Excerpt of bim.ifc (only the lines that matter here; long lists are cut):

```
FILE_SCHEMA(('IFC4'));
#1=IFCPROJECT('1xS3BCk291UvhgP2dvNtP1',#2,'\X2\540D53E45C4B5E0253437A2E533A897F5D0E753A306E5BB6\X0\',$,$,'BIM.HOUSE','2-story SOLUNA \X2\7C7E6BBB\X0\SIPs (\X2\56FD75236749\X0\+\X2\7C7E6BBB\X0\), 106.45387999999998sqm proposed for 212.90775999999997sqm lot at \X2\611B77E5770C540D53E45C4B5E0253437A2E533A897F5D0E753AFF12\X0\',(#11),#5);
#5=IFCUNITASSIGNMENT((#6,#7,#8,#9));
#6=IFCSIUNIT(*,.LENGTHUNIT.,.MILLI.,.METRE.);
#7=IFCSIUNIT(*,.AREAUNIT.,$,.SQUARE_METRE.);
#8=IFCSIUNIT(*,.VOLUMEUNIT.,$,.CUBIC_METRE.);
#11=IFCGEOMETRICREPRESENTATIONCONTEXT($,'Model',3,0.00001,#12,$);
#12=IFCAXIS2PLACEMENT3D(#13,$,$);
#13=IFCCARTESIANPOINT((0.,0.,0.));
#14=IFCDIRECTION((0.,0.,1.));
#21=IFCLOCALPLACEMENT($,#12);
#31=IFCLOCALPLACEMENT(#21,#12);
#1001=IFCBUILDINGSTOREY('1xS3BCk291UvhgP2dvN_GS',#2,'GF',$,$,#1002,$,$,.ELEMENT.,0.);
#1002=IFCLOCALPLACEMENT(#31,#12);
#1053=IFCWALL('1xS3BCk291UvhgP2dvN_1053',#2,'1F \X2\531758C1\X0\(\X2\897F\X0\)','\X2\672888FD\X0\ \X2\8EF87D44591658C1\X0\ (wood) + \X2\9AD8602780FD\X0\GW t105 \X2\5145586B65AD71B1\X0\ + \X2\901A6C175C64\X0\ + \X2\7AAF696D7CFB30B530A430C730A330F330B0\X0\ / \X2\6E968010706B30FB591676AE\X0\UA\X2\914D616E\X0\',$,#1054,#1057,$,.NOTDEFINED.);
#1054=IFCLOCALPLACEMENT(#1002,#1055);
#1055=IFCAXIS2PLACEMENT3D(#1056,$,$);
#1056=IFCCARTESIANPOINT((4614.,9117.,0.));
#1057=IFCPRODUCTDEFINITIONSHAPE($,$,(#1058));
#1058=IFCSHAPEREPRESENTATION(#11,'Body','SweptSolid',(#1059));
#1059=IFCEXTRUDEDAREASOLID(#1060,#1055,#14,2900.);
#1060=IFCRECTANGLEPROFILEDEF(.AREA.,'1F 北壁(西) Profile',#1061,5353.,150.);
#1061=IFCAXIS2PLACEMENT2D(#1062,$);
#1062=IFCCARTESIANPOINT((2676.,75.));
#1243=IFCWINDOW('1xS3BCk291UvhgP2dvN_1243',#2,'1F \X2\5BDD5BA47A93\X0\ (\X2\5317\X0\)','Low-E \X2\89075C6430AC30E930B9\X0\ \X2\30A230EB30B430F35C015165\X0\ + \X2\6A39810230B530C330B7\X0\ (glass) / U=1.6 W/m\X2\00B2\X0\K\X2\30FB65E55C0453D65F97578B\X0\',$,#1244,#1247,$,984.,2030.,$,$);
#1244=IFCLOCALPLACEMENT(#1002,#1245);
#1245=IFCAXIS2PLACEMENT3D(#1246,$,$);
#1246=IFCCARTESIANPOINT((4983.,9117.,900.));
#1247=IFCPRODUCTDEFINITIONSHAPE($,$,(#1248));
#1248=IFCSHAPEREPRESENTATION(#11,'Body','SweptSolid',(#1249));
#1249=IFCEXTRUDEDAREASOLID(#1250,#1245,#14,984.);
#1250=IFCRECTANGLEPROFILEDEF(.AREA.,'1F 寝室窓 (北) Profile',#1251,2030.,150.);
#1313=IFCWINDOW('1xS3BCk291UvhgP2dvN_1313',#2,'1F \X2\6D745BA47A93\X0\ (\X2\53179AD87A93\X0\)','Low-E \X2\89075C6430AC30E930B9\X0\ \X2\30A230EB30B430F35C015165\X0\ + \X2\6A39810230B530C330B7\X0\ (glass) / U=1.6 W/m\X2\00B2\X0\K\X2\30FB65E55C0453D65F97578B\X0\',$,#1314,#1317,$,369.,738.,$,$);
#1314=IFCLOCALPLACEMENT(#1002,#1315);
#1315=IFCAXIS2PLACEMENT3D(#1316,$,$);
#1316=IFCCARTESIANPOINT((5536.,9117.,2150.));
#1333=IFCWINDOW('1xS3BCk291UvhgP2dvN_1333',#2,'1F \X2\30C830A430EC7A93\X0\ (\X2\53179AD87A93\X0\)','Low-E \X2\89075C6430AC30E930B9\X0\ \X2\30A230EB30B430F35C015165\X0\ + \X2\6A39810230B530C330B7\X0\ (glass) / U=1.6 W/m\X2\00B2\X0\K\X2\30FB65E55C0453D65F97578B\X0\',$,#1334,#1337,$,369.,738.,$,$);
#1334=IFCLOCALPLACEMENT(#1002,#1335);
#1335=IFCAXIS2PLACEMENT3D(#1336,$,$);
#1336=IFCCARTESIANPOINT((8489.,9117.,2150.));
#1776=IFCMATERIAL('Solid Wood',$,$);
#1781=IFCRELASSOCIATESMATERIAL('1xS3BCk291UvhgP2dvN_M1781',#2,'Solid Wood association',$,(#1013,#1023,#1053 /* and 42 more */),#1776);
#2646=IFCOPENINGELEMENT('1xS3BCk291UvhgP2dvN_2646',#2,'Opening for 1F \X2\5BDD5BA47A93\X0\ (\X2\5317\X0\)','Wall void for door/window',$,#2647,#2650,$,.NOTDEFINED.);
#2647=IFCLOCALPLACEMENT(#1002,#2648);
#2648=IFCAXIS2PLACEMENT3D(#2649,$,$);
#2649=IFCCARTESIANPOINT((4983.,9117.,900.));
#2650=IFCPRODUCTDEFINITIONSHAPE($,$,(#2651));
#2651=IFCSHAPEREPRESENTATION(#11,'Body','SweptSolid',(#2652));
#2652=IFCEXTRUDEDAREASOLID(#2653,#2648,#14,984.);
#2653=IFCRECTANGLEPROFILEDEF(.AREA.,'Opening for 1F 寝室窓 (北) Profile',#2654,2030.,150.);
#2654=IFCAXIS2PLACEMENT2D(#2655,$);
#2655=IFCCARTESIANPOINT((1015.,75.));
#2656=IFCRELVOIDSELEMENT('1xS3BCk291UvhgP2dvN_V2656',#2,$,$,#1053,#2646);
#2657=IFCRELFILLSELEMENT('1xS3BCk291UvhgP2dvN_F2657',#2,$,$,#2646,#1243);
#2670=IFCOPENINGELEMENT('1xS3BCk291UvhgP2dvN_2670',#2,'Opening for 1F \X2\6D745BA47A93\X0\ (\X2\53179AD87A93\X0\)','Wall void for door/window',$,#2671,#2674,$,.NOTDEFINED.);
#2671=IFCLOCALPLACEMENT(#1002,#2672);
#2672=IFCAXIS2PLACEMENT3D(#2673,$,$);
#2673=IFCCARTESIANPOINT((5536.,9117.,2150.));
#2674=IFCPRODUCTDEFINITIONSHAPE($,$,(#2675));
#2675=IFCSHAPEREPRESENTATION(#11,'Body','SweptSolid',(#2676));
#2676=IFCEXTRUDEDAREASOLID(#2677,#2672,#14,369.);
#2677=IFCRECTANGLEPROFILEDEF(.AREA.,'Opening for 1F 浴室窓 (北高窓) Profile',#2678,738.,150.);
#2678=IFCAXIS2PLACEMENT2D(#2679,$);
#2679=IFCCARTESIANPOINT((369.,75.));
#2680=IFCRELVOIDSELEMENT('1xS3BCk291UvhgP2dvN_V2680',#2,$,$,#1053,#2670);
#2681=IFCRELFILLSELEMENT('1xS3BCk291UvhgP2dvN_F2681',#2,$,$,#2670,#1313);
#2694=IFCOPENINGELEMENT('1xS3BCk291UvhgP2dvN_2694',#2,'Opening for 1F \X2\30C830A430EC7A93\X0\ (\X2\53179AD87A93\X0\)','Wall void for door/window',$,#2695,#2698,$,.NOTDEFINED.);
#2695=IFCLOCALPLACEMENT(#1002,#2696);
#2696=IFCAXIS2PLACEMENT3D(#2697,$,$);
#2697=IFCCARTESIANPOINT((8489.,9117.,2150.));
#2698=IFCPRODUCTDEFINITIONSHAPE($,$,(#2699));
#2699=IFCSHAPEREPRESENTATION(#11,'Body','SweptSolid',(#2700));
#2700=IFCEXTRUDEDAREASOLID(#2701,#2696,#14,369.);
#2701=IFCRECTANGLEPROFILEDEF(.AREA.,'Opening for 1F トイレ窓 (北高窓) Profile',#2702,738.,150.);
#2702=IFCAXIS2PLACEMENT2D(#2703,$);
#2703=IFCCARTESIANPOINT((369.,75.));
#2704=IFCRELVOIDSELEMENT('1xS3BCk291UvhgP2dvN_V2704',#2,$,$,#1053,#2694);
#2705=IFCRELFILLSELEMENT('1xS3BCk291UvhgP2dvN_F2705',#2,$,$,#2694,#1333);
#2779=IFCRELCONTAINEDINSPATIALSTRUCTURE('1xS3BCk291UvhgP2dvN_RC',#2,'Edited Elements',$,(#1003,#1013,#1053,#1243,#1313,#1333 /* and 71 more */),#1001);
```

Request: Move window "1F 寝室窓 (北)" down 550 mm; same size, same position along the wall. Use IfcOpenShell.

```python
import numpy as np
import ifcopenshell
import ifcopenshell.api.geometry
import ifcopenshell.util.placement
import ifcopenshell.util.unit

model = ifcopenshell.open("bim.ifc")
unit_scale = ifcopenshell.util.unit.calculate_unit_scale(model)

window = model.by_guid("1xS3BCk291UvhgP2dvN_1243")
opening = window.FillsVoids[0].RelatingOpeningElement
dz = -0.55 / unit_scale

shift = np.array([0.0, 0.0, dz])
# The window is not placed relative to its opening, so move both.
for product in (opening, window):
    matrix = ifcopenshell.util.placement.get_local_placement(product.ObjectPlacement)
    matrix[:3, 3] += shift
    ifcopenshell.api.geometry.edit_object_placement(model, product=product, matrix=matrix, is_si=False)

print(f"moved by {dz * unit_scale:+.3f} m")

model.write("bim_v2.ifc")
```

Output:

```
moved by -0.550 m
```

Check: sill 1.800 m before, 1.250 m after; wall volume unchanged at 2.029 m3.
